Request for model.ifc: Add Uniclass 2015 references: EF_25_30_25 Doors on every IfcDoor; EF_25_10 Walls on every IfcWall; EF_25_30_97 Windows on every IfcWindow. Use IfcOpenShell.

First a look at what the model holds.

```python
import ifcopenshell

model = ifcopenshell.open("model.ifc")
print(model.schema)
print("classifications:", [c.Name for c in model.by_type("IfcClassification")])
for ifc_class in ("IfcDoor", "IfcRoof", "IfcStair", "IfcWall", "IfcWindow"):
    print(ifc_class, len(model.by_type(ifc_class)))
```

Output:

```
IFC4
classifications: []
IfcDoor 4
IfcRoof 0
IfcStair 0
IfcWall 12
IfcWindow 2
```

```python
import ifcopenshell
import ifcopenshell.api.classification

model = ifcopenshell.open("model.ifc")

system = ifcopenshell.api.classification.add_classification(model, classification="Uniclass 2015")

codes = {
    "IfcDoor": ("EF_25_30_25", "Doors"),
    "IfcWall": ("EF_25_10", "Walls"),
    "IfcWindow": ("EF_25_30_97", "Windows"),
}
for ifc_class, (code, name) in codes.items():
    products = model.by_type(ifc_class)
    ifcopenshell.api.classification.add_reference(
        model, products=products, classification=system, identification=code, name=name
    )
    print(code, len(products))

model.write("model_updated.ifc")
```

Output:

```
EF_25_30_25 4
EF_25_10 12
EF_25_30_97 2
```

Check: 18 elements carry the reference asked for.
